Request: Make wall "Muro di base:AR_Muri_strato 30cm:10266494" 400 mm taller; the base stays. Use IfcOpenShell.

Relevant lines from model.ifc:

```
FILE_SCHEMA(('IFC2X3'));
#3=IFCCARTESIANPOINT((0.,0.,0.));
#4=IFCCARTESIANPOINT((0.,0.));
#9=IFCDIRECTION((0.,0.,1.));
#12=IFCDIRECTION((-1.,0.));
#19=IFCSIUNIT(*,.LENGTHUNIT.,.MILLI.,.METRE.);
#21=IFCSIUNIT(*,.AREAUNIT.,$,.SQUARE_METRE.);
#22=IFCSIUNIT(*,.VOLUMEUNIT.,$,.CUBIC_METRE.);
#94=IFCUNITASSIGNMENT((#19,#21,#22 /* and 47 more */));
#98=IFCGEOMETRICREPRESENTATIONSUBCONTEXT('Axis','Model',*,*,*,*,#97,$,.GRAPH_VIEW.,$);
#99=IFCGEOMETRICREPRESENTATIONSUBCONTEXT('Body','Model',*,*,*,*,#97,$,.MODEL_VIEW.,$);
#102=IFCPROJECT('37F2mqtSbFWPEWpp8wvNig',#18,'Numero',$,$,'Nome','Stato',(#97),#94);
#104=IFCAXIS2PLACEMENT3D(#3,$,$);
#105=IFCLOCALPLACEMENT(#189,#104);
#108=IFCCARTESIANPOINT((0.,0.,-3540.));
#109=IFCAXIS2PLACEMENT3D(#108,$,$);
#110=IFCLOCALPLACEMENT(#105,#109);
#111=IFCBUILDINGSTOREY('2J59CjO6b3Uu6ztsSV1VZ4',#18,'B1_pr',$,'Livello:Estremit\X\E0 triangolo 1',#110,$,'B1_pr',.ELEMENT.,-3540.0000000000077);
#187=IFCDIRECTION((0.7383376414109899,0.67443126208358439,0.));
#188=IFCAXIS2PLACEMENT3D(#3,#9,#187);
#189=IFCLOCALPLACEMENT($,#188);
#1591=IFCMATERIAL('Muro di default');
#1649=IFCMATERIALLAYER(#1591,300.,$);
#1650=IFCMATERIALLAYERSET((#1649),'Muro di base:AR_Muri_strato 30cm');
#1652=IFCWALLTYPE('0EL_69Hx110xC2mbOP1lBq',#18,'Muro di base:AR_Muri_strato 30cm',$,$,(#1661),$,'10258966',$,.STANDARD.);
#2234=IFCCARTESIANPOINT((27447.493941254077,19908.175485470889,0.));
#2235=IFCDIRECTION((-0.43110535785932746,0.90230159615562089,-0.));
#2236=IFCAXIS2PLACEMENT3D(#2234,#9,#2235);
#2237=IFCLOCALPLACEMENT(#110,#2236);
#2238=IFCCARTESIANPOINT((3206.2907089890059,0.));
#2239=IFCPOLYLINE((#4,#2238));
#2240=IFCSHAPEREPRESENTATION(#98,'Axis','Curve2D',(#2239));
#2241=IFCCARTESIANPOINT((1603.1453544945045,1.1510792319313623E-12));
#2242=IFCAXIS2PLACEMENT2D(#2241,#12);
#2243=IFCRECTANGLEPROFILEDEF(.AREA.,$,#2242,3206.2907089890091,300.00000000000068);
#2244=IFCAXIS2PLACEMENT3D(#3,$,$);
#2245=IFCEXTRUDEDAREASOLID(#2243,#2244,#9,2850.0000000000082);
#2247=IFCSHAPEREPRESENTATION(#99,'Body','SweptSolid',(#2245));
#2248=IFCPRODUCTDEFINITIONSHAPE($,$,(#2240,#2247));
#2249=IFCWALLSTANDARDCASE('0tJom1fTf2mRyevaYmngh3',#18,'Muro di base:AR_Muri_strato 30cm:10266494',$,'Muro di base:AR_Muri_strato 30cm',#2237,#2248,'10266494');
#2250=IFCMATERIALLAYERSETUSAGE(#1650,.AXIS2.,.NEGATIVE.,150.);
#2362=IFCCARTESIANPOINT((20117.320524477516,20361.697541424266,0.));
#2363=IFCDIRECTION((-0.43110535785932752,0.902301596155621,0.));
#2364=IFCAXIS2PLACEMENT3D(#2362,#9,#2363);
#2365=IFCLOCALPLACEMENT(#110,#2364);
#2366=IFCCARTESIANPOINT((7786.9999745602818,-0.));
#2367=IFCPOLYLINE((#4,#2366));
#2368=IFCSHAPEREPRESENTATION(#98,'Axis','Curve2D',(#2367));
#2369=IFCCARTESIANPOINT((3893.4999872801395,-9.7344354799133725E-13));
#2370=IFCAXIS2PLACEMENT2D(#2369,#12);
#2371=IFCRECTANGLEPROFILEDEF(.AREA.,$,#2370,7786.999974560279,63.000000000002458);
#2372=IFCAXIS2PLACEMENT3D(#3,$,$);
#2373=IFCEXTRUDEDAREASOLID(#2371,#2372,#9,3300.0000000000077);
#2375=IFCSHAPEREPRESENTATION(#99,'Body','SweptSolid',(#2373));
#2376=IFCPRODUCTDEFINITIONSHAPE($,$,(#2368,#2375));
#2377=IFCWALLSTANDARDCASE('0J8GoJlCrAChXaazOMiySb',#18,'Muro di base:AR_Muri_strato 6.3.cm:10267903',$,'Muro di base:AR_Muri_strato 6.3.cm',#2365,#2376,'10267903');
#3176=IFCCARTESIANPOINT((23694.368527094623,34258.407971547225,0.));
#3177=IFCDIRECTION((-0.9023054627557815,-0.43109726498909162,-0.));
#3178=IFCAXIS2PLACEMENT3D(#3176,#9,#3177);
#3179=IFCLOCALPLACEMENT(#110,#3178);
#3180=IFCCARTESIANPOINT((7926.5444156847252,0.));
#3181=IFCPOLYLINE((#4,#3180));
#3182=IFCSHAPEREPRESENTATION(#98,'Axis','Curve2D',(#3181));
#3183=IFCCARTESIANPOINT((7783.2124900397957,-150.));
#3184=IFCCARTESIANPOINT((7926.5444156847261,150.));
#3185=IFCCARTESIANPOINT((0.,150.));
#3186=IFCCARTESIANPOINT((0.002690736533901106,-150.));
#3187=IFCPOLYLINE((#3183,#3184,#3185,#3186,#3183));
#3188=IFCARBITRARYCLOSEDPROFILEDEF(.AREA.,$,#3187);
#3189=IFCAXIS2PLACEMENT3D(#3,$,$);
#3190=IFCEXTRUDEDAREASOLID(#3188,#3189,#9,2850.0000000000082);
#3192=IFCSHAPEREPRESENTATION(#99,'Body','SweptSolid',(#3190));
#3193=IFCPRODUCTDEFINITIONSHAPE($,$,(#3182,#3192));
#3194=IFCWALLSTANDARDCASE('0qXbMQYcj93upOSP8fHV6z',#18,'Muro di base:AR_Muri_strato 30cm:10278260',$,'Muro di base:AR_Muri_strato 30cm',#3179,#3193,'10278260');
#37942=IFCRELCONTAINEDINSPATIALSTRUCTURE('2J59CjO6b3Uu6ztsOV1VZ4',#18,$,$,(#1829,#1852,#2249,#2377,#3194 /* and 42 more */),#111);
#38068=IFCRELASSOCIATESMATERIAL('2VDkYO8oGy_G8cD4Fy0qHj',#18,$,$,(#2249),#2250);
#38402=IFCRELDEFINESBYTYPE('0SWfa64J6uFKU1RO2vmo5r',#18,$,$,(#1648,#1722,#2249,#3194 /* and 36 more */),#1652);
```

```python
import ifcopenshell
import ifcopenshell.geom
import ifcopenshell.util.representation
import ifcopenshell.util.shape

model = ifcopenshell.open("model.ifc")
settings = ifcopenshell.geom.settings()


def volume(element):
    """Net volume in cubic metres, openings subtracted."""
    shape = ifcopenshell.geom.create_shape(settings, element)
    return ifcopenshell.util.shape.get_volume(shape.geometry)


wall = model.by_id(2249)
before = volume(wall)

body = ifcopenshell.util.representation.get_representation(wall, "Model", "Body")
solid = body.Items[0]
old_height = solid.Depth
solid.Depth += 400.0
after = volume(wall)

print(f"height {old_height:g} -> {solid.Depth:g}, volume {before:.3f} -> {after:.3f} m3")

model.write("model_v2.ifc")
```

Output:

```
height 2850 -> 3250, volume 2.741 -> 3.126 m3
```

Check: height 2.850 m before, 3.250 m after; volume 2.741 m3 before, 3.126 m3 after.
